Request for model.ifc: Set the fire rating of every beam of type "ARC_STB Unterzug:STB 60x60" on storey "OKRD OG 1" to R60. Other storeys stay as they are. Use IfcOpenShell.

First a look at what the model holds.

```python
import ifcopenshell
import ifcopenshell.util.element

model = ifcopenshell.open("model.ifc")
print(model.schema)
storey = next(s for s in model.by_type("IfcBuildingStorey") if s.Name == "OKRD OG 1")
beams = [e for e in ifcopenshell.util.element.get_decomposition(storey) if e.is_a("IfcBeam")]
seen = {}
for e in beams:
    element_type = ifcopenshell.util.element.get_type(e)
    key = (element_type.Name if element_type != e and element_type else None, ifcopenshell.util.element.get_pset(e, "Pset_BeamCommon", "FireRating"))
    seen[key] = seen.get(key, 0) + 1
for (name, value), count in sorted(seen.items(), key=str):
    print(count, "x", name, "|", value)
```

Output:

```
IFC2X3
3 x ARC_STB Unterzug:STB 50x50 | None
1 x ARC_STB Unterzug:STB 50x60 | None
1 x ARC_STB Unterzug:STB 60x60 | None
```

```python
import ifcopenshell
import ifcopenshell.api.pset
import ifcopenshell.util.element

model = ifcopenshell.open("model.ifc")

storey = next(s for s in model.by_type("IfcBuildingStorey") if s.Name == "OKRD OG 1")
beams = [e for e in ifcopenshell.util.element.get_decomposition(storey) if e.is_a("IfcBeam")]

count = 0
for e in beams:
    element_type = ifcopenshell.util.element.get_type(e)
    if element_type in (None, e) or element_type.Name != "ARC_STB Unterzug:STB 60x60":
        continue
    # add_pset returns the element's existing set when there is one.
    pset = ifcopenshell.api.pset.add_pset(model, product=e, name="Pset_BeamCommon")
    ifcopenshell.api.pset.edit_pset(model, pset=pset, properties={"FireRating": "R60"})
    count += 1

print(count, "beams updated")

model.write("model_edited.ifc")
```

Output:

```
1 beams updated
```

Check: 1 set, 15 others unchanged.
